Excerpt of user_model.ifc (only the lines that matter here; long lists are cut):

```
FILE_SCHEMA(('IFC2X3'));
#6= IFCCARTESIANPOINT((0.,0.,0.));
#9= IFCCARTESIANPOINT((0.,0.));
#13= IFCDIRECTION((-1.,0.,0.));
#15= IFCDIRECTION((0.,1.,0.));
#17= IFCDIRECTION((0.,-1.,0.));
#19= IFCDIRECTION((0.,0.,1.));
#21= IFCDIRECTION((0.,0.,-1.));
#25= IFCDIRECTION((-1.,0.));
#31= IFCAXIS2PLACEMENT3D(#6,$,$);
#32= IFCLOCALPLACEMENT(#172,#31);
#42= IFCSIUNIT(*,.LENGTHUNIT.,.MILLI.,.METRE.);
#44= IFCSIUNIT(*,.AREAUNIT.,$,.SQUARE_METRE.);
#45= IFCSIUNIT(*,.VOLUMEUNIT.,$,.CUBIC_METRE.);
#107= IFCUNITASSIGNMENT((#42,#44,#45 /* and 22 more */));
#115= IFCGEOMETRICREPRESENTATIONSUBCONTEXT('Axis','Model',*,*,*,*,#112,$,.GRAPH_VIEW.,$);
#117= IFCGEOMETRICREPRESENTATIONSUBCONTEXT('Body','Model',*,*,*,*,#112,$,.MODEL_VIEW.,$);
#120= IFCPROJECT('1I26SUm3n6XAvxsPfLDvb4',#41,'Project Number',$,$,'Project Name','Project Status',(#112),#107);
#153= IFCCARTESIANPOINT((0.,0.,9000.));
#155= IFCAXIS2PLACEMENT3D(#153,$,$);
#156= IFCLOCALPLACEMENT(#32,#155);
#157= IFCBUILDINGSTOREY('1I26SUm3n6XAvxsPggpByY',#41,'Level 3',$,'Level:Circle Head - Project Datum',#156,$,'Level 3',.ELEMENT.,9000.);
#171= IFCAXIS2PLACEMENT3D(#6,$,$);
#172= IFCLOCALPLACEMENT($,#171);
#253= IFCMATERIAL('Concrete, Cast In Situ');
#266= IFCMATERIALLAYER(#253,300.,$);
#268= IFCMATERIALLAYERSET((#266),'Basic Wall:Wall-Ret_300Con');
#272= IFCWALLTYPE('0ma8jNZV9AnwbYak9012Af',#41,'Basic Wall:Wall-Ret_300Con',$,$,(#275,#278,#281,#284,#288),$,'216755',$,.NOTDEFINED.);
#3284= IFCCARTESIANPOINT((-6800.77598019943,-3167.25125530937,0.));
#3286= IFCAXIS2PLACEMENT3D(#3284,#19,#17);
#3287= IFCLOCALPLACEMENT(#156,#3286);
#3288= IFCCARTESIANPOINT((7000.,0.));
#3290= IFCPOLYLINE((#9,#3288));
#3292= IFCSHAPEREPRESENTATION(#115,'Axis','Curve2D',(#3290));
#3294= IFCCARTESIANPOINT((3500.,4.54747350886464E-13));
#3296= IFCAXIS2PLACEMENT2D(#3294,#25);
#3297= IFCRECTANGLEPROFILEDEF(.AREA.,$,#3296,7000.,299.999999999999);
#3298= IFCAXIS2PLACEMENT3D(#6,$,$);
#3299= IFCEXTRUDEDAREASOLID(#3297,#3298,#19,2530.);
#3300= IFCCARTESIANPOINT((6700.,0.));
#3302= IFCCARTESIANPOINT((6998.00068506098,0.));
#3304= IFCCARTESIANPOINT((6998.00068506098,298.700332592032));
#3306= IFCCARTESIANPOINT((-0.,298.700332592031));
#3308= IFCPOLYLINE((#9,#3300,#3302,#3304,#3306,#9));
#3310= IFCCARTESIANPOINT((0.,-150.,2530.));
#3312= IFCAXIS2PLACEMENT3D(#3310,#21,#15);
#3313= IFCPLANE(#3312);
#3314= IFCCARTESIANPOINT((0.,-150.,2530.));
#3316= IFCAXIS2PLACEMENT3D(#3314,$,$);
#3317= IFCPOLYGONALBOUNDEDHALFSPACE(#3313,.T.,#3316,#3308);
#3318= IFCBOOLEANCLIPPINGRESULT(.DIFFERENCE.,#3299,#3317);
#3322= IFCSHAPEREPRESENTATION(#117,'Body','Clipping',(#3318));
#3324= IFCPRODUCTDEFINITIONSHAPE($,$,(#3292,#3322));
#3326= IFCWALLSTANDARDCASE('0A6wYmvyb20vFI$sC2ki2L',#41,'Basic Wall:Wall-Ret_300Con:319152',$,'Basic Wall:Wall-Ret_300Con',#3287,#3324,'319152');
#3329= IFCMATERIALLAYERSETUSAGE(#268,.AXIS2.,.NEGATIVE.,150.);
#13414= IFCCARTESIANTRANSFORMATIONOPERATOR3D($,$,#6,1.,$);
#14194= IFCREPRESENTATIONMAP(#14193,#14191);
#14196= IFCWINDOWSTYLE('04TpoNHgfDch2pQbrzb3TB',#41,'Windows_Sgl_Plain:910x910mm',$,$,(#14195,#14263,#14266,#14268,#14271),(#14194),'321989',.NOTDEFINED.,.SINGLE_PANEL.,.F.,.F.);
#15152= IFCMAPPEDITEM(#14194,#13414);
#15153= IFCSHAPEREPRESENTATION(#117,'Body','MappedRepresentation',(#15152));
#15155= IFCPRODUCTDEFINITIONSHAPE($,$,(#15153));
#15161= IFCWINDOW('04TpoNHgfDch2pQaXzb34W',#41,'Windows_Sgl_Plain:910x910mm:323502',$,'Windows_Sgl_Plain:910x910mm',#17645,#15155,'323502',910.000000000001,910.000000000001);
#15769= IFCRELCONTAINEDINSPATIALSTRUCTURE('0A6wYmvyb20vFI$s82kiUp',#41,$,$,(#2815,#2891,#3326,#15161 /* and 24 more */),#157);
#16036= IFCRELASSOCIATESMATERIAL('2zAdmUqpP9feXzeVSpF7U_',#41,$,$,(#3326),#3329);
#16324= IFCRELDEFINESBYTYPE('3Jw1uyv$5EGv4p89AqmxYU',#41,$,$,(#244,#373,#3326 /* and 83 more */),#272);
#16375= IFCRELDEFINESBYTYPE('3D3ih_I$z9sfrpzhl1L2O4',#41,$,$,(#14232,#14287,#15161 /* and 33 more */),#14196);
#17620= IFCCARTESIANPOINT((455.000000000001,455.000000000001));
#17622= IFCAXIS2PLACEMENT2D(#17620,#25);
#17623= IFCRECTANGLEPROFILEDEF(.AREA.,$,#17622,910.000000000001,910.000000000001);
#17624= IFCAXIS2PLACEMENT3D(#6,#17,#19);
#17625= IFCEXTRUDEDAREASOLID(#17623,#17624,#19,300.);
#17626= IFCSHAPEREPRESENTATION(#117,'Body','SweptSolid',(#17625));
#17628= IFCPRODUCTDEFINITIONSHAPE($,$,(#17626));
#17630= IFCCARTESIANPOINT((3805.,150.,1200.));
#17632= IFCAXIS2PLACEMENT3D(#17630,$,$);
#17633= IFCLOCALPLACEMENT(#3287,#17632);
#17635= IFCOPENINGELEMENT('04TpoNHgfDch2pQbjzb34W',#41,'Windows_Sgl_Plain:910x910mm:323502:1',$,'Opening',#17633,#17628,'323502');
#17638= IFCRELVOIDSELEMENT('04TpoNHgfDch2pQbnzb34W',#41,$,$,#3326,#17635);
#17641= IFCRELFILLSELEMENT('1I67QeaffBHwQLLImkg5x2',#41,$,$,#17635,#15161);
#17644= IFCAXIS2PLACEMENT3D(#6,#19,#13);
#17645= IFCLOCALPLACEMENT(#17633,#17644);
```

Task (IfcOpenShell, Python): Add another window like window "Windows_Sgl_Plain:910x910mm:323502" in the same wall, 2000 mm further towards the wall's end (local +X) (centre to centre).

```python
import ifcopenshell
import ifcopenshell.api.feature
import ifcopenshell.api.geometry
import ifcopenshell.api.root
import ifcopenshell.geom
import ifcopenshell.util.element
import ifcopenshell.util.placement
import ifcopenshell.util.shape
import ifcopenshell.util.unit

model = ifcopenshell.open("user_model.ifc")
unit_scale = ifcopenshell.util.unit.calculate_unit_scale(model)
settings = ifcopenshell.geom.settings()


def volume(element):
    """Net volume in cubic metres, openings subtracted."""
    shape = ifcopenshell.geom.create_shape(settings, element)
    return ifcopenshell.util.shape.get_volume(shape.geometry)


def reuse_history(source, copy):
    """copy_class also copies each property set's owner history, people and application; keep the originals."""
    for rel in copy.IsDefinedBy:
        if rel.is_a("IfcRelDefinesByProperties") and (history := rel.RelatingPropertyDefinition.OwnerHistory):
            rel.RelatingPropertyDefinition.OwnerHistory = source.OwnerHistory
            ifcopenshell.util.element.remove_deep2(model, history)


window = model.by_guid("04TpoNHgfDch2pQaXzb34W")
opening = window.FillsVoids[0].RelatingOpeningElement
wall = opening.VoidsElements[0].RelatingBuildingElement
before = volume(wall)
shift = ifcopenshell.util.placement.get_local_placement(wall.ObjectPlacement)[:3, 0] * 2 / unit_scale

# copy_class copies the void relationship, type, container and properties, but no geometry.
new_opening = ifcopenshell.api.root.copy_class(model, product=opening)
new_opening.Representation = ifcopenshell.util.element.copy_deep(
    model, opening.Representation, exclude=["IfcGeometricRepresentationContext", "IfcRepresentationMap"]
)
new_opening.Name = "Windows_Sgl_Plain:910x910mm"
new_opening.Tag = None
new_window = ifcopenshell.api.root.copy_class(model, product=window)
new_window.Representation = ifcopenshell.util.element.copy_deep(
    model, window.Representation, exclude=["IfcGeometricRepresentationContext", "IfcRepresentationMap"]
)
new_window.Name = "Windows_Sgl_Plain:910x910mm"
new_window.Tag = None
reuse_history(window, new_window)
fills = ifcopenshell.api.feature.add_filling(model, opening=new_opening, element=new_window)
fills.OwnerHistory = new_window.OwnerHistory  # required in IFC2X3

for old, new in ((opening, new_opening), (window, new_window)):
    matrix = ifcopenshell.util.placement.get_local_placement(old.ObjectPlacement)
    matrix[:3, 3] += shift
    ifcopenshell.api.geometry.edit_object_placement(model, product=new, matrix=matrix, is_si=False)

after = volume(wall)

print(f"wall volume {before:.3f} -> {after:.3f} m3")

model.write("user_model_edited.ifc")
```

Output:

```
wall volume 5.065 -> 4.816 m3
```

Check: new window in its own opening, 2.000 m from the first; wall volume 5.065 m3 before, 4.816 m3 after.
